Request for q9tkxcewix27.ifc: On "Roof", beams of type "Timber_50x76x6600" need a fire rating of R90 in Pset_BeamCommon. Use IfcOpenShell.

First a look at what the model holds.

```python
import ifcopenshell
import ifcopenshell.util.element

model = ifcopenshell.open("q9tkxcewix27.ifc")
print(model.schema)
storey = next(s for s in model.by_type("IfcBuildingStorey") if s.Name == "Roof")
beams = [e for e in ifcopenshell.util.element.get_decomposition(storey) if e.is_a("IfcBeam")]
seen = {}
for e in beams:
    element_type = ifcopenshell.util.element.get_type(e)
    key = (element_type.Name if element_type != e and element_type else None, ifcopenshell.util.element.get_pset(e, "Pset_BeamCommon", "FireRating"))
    seen[key] = seen.get(key, 0) + 1
for (name, value), count in sorted(seen.items(), key=str):
    print(count, "x", name, "|", value)
```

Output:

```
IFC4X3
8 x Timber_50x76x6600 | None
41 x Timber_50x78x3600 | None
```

```python
import ifcopenshell
import ifcopenshell.api.pset
import ifcopenshell.util.element

model = ifcopenshell.open("q9tkxcewix27.ifc")

storey = next(s for s in model.by_type("IfcBuildingStorey") if s.Name == "Roof")
beams = [e for e in ifcopenshell.util.element.get_decomposition(storey) if e.is_a("IfcBeam")]

count = 0
for e in beams:
    element_type = ifcopenshell.util.element.get_type(e)
    if element_type in (None, e) or element_type.Name != "Timber_50x76x6600":
        continue
    # add_pset returns the element's existing set when there is one.
    pset = ifcopenshell.api.pset.add_pset(model, product=e, name="Pset_BeamCommon")
    ifcopenshell.api.pset.edit_pset(model, pset=pset, properties={"FireRating": "R90"})
    count += 1

print(count, "beams updated")

model.write("q9tkxcewix27-out.ifc")
```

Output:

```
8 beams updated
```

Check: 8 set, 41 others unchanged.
